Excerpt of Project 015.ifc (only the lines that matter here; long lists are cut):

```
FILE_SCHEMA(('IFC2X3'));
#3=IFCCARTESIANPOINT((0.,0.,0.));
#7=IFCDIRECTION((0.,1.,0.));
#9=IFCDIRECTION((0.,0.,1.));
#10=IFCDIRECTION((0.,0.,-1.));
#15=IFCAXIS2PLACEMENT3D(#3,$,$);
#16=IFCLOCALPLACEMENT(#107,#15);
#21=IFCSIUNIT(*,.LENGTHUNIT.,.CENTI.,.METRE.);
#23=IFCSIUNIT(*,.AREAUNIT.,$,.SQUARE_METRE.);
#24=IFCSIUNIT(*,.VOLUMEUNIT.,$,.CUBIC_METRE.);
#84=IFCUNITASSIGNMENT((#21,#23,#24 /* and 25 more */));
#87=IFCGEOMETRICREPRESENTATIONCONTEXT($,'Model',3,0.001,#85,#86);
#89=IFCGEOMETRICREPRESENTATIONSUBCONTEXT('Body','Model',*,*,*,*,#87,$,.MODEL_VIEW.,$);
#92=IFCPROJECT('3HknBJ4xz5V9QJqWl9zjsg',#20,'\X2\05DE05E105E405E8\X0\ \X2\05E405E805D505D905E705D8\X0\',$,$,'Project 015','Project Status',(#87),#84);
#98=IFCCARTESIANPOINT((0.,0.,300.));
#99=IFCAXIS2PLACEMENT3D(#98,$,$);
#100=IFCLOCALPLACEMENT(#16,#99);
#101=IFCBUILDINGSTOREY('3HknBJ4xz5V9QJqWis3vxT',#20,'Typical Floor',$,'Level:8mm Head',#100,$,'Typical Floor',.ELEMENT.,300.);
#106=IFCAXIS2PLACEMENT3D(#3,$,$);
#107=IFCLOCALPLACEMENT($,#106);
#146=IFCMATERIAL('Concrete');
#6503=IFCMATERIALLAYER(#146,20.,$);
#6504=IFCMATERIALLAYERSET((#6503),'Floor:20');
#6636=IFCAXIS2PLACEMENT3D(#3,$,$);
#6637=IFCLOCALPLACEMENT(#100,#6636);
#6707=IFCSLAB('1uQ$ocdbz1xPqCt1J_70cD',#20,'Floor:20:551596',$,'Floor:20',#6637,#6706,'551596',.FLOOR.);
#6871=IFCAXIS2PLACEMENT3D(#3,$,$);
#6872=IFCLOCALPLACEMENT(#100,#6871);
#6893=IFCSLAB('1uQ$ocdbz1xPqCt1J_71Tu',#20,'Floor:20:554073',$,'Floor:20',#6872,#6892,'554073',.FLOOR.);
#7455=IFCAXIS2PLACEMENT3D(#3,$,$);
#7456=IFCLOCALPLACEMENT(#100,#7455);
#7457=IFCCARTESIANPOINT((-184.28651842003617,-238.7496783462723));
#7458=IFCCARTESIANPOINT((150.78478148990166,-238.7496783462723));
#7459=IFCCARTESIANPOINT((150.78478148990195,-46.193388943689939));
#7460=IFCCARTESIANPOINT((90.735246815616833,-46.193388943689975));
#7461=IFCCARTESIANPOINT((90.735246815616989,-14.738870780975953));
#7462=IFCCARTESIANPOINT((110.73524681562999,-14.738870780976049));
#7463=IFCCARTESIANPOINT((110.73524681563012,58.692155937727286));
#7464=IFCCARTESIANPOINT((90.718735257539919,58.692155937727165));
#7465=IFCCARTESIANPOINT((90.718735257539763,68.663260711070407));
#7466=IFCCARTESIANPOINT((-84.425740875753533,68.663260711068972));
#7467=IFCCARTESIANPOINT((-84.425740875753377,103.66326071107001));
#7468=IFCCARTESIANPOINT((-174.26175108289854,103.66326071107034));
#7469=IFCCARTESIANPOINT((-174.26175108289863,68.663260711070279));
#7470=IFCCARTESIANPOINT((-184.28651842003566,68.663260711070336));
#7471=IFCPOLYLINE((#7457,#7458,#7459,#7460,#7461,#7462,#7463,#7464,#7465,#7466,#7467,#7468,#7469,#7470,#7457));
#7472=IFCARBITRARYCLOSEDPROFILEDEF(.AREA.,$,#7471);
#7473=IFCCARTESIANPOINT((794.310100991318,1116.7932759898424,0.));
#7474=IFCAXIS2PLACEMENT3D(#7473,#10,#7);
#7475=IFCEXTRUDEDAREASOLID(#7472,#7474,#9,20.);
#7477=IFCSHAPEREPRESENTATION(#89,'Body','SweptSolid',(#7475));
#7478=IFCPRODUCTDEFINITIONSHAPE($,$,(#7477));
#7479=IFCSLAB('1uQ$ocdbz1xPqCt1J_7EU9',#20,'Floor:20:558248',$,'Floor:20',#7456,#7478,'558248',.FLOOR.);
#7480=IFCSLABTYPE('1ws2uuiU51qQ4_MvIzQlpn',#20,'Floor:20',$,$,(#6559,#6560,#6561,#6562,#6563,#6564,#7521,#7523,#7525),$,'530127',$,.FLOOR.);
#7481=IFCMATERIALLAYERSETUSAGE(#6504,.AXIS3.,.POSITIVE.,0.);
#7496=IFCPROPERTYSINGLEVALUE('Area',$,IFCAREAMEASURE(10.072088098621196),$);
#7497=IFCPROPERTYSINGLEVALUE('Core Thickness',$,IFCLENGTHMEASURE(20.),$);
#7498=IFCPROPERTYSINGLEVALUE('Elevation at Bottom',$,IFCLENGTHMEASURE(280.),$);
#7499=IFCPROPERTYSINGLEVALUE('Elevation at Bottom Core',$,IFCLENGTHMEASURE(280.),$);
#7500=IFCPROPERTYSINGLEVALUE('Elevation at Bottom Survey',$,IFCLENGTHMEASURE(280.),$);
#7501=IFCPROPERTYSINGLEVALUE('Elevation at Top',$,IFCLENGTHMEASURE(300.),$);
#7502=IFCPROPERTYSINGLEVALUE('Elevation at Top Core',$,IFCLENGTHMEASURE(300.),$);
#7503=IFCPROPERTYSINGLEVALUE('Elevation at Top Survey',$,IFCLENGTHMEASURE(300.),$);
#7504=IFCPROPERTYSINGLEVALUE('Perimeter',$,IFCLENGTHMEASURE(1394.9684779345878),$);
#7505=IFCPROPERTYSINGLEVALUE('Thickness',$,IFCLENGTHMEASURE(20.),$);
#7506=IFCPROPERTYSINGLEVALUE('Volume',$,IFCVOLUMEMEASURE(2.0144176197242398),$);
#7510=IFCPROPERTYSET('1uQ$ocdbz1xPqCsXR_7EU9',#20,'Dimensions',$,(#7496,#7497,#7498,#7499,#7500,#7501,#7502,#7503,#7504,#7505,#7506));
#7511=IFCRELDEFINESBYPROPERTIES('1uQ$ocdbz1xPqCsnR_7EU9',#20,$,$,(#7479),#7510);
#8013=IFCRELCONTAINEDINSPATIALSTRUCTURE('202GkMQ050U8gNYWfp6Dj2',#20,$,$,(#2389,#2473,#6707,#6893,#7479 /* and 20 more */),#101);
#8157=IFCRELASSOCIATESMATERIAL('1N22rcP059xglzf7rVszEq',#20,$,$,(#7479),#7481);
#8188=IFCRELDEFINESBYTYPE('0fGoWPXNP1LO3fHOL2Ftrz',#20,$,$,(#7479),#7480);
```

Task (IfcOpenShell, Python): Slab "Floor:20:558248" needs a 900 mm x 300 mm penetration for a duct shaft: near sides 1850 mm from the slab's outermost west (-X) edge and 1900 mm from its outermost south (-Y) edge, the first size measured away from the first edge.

```python
import numpy as np
import ifcopenshell
import ifcopenshell.api.feature
import ifcopenshell.api.geometry
import ifcopenshell.api.pset
import ifcopenshell.api.root
import ifcopenshell.geom
import ifcopenshell.util.element
import ifcopenshell.util.placement
import ifcopenshell.util.representation
import ifcopenshell.util.shape
import ifcopenshell.util.unit

model = ifcopenshell.open("Project 015.ifc")
unit_scale = ifcopenshell.util.unit.calculate_unit_scale(model)
area_scale = ifcopenshell.util.unit.calculate_unit_scale(model, "AREAUNIT")
volume_scale = ifcopenshell.util.unit.calculate_unit_scale(model, "VOLUMEUNIT")
settings = ifcopenshell.geom.settings()


def volume(element):
    """Net volume in cubic metres, openings subtracted."""
    shape = ifcopenshell.geom.create_shape(settings, element)
    return ifcopenshell.util.shape.get_volume(shape.geometry)


slab = model.by_guid("1uQ$ocdbz1xPqCt1J_7EU9")
before = volume(slab)

# Extent in the slab's own axes, in metres. The edges named are its -X and -Y sides.
slab_shape = ifcopenshell.geom.create_shape(settings, slab)
vertices = ifcopenshell.util.shape.get_vertices(slab_shape.geometry)
x_min, y_min, bottom = vertices.min(axis=0)
top = vertices[:, 2].max()

opening = ifcopenshell.api.root.create_entity(model, ifc_class="IfcOpeningElement", name="Duct shaft opening")
context = ifcopenshell.util.representation.get_context(model, "Model", "Body", "MODEL_VIEW")
width, depth = 0.9, 0.3
outline = [(0.0, 0.0), (width, 0.0), (width, depth), (0.0, depth), (0.0, 0.0)]
# Overshoot both faces by 50 mm so the cut is clean.
shape = ifcopenshell.api.geometry.add_slab_representation(
    model, context=context, depth=top - bottom + 0.1, polyline=outline
)
ifcopenshell.api.geometry.assign_representation(model, product=opening, representation=shape)

matrix = ifcopenshell.util.placement.get_local_placement(slab.ObjectPlacement)
matrix[:, 3] = matrix @ np.append(np.array([x_min + 1.85, y_min + 1.9, bottom - 0.05]) / unit_scale, 1.0)
ifcopenshell.api.geometry.edit_object_placement(model, product=opening, matrix=matrix, is_si=False)
ifcopenshell.api.feature.add_feature(model, feature=opening, element=slab)

after = volume(slab)

# Update the slab's stored quantities.
pset = model.by_id(ifcopenshell.util.element.get_pset(slab, "Dimensions", should_inherit=False)["id"])
ifcopenshell.api.pset.edit_pset(model, pset=pset, properties={
    "Area": model.create_entity("IfcAreaMeasure", after / (top - bottom) / area_scale),
    "Volume": model.create_entity("IfcVolumeMeasure", after / volume_scale),
})

print(f"slab volume {before:.3f} -> {after:.3f} m3")

model.write("Project 015_edited.ifc")
```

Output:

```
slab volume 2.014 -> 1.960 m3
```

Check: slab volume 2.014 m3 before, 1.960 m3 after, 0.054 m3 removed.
